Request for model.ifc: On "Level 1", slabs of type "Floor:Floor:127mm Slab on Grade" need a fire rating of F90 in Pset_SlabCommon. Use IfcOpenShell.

First a look at what the model holds.

```python
import ifcopenshell
import ifcopenshell.util.element

model = ifcopenshell.open("model.ifc")
print(model.schema)
storey = next(s for s in model.by_type("IfcBuildingStorey") if s.Name == "Level 1")
slabs = [e for e in ifcopenshell.util.element.get_decomposition(storey) if e.is_a("IfcSlab")]
seen = {}
for e in slabs:
    element_type = ifcopenshell.util.element.get_type(e)
    key = (element_type.Name if element_type != e and element_type else None, ifcopenshell.util.element.get_pset(e, "Pset_SlabCommon", "FireRating"))
    seen[key] = seen.get(key, 0) + 1
for (name, value), count in sorted(seen.items(), key=str):
    print(count, "x", name, "|", value)
```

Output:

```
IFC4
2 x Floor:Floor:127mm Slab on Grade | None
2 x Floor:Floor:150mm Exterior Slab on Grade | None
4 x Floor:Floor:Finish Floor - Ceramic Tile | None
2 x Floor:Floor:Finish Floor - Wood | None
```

```python
import ifcopenshell
import ifcopenshell.api.pset
import ifcopenshell.util.element

model = ifcopenshell.open("model.ifc")

storey = next(s for s in model.by_type("IfcBuildingStorey") if s.Name == "Level 1")
slabs = [e for e in ifcopenshell.util.element.get_decomposition(storey) if e.is_a("IfcSlab")]

count = 0
for e in slabs:
    element_type = ifcopenshell.util.element.get_type(e)
    if element_type in (None, e) or element_type.Name != "Floor:Floor:127mm Slab on Grade":
        continue
    # add_pset returns the element's existing set when there is one.
    pset = ifcopenshell.api.pset.add_pset(model, product=e, name="Pset_SlabCommon")
    ifcopenshell.api.pset.edit_pset(model, pset=pset, properties={"FireRating": "F90"})
    count += 1

print(count, "slabs updated")

model.write("model_rev.ifc")
```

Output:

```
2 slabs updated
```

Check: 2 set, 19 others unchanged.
